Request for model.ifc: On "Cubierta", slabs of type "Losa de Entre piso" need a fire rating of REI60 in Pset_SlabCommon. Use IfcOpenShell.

First a look at what the model holds.

```python
import ifcopenshell
import ifcopenshell.util.element

model = ifcopenshell.open("model.ifc")
print(model.schema)
storey = next(s for s in model.by_type("IfcBuildingStorey") if s.Name == "Cubierta")
slabs = [e for e in ifcopenshell.util.element.get_decomposition(storey) if e.is_a("IfcSlab")]
seen = {}
for e in slabs:
    element_type = ifcopenshell.util.element.get_type(e)
    key = (element_type.Name if element_type != e and element_type else None, ifcopenshell.util.element.get_pset(e, "Pset_SlabCommon", "FireRating"))
    seen[key] = seen.get(key, 0) + 1
for (name, value), count in sorted(seen.items(), key=str):
    print(count, "x", name, "|", value)
```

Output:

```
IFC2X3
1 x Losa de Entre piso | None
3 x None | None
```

```python
import ifcopenshell
import ifcopenshell.api.pset
import ifcopenshell.util.element

model = ifcopenshell.open("model.ifc")

storey = next(s for s in model.by_type("IfcBuildingStorey") if s.Name == "Cubierta")
slabs = [e for e in ifcopenshell.util.element.get_decomposition(storey) if e.is_a("IfcSlab")]

count = 0
for e in slabs:
    element_type = ifcopenshell.util.element.get_type(e)
    if element_type in (None, e) or element_type.Name != "Losa de Entre piso":
        continue
    # add_pset returns the element's existing set when there is one.
    pset = ifcopenshell.api.pset.add_pset(model, product=e, name="Pset_SlabCommon")
    ifcopenshell.api.pset.edit_pset(model, pset=pset, properties={"FireRating": "REI60"})
    count += 1

print(count, "slabs updated")

model.write("model_v2.ifc")
```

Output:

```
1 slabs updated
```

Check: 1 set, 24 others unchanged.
